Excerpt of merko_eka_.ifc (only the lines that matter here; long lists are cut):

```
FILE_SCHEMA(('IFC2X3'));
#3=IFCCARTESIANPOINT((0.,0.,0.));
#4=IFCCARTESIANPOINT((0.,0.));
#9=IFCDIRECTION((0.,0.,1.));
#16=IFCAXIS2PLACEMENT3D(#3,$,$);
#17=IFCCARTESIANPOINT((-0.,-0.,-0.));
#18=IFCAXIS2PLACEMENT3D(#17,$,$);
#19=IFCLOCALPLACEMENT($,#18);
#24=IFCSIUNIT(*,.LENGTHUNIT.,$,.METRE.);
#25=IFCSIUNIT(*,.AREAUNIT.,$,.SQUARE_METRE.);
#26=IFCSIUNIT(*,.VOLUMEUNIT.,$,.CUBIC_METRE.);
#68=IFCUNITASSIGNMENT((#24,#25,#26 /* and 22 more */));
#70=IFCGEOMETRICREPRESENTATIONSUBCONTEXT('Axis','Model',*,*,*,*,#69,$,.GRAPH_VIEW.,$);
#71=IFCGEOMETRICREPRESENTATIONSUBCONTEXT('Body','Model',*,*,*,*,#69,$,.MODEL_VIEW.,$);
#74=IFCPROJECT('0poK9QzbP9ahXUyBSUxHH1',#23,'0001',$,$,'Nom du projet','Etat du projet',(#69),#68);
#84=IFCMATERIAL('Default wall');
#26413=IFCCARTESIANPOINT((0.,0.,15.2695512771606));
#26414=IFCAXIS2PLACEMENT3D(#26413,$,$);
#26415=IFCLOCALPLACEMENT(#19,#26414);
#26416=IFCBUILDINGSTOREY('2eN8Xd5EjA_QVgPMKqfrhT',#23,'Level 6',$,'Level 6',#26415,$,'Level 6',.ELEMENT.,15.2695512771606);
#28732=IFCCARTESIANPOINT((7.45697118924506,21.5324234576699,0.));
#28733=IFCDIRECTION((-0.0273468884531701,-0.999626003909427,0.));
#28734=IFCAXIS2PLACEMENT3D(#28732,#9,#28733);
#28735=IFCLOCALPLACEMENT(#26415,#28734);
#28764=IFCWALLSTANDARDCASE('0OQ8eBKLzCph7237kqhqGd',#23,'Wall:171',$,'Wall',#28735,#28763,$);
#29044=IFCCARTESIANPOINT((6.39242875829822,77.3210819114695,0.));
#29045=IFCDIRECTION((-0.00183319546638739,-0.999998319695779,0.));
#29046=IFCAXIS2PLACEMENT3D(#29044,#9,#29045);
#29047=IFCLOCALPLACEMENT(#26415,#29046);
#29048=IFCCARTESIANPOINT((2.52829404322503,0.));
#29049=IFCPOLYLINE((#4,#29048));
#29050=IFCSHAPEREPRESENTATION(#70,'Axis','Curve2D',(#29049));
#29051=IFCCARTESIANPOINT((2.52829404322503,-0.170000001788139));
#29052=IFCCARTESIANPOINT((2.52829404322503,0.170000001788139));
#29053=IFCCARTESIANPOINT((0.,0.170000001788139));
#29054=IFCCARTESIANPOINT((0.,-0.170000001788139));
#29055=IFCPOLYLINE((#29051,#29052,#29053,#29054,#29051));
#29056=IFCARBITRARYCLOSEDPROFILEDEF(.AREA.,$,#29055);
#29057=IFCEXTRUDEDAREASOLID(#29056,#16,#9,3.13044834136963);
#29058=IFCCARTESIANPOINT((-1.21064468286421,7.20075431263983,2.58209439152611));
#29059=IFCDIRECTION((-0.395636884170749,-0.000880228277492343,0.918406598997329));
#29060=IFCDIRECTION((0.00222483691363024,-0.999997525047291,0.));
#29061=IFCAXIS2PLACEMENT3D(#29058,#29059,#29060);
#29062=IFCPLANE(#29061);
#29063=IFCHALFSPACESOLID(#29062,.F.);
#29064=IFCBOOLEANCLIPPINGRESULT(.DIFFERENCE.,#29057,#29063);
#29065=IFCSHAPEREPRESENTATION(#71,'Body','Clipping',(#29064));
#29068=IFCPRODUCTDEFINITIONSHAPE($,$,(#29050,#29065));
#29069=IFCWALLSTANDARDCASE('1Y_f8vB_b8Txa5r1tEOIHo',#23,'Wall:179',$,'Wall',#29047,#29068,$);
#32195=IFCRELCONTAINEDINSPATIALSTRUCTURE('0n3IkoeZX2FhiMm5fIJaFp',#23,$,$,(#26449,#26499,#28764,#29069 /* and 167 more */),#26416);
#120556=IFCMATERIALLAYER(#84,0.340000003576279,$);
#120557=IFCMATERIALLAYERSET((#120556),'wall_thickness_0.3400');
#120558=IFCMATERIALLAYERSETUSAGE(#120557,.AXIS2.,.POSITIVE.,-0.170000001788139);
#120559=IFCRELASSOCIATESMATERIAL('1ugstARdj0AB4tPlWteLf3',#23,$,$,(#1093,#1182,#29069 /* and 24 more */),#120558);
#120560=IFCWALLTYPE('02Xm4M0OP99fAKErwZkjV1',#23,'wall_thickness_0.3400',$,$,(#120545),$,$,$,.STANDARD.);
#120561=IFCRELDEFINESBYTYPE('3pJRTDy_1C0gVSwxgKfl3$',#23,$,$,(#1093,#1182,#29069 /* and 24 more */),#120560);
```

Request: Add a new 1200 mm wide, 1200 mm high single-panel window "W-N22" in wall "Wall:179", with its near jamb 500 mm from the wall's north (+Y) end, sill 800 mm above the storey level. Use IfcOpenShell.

```python
import numpy as np
import ifcopenshell
import ifcopenshell.api.feature
import ifcopenshell.api.geometry
import ifcopenshell.api.root
import ifcopenshell.api.spatial
import ifcopenshell.api.type
import ifcopenshell.geom
import ifcopenshell.util.element
import ifcopenshell.util.placement
import ifcopenshell.util.representation
import ifcopenshell.util.shape
import ifcopenshell.util.unit

model = ifcopenshell.open("merko_eka_.ifc")
unit_scale = ifcopenshell.util.unit.calculate_unit_scale(model)
settings = ifcopenshell.geom.settings()


def volume(element):
    """Net volume in cubic metres, openings subtracted."""
    shape = ifcopenshell.geom.create_shape(settings, element)
    return ifcopenshell.util.shape.get_volume(shape.geometry)


wall = model.by_guid("1Y_f8vB_b8Txa5r1tEOIHo")
storey = ifcopenshell.util.element.get_container(wall, ifc_class="IfcBuildingStorey")
context = ifcopenshell.util.representation.get_context(model, "Model", "Body", "MODEL_VIEW")
before = volume(wall)

width, height, from_end, sill = 1.2, 1.2, 0.5, 0.8  # metres

# The wall runs along its own X axis, and the end named is its -X end.
wall_shape = ifcopenshell.geom.create_shape(settings, wall)
x, y, z = ifcopenshell.util.shape.get_vertices(wall_shape.geometry).T
start = x.min() + from_end
face, thickness = float(y.min()), float(y.max() - y.min())
wall_matrix = ifcopenshell.util.placement.get_local_placement(wall.ObjectPlacement)
level = ifcopenshell.util.placement.get_local_placement(storey.ObjectPlacement)[2, 3]


def in_wall(x, y):
    """Placement at x, y metres in the wall's axes, at sill height."""
    matrix = wall_matrix.copy()
    matrix[:, 3] = wall_matrix @ np.array([x / unit_scale, y / unit_scale, 0.0, 1.0])
    matrix[2, 3] = level + sill / unit_scale
    return matrix


# Opening: a box that overshoots both wall faces by 50 mm.
opening = ifcopenshell.api.root.create_entity(model, ifc_class="IfcOpeningElement")
box = ifcopenshell.api.geometry.add_wall_representation(
    model, context=context, length=width, height=height, thickness=thickness + 0.1
)
ifcopenshell.api.geometry.assign_representation(model, product=opening, representation=box)
ifcopenshell.api.geometry.edit_object_placement(model, product=opening, matrix=in_wall(start, face - 0.05), is_si=False)
ifcopenshell.api.feature.add_feature(model, feature=opening, element=wall)

window = ifcopenshell.api.root.create_entity(model, ifc_class="IfcWindow", name="W-N22")
window.OverallWidth, window.OverallHeight = width / unit_scale, height / unit_scale
body = ifcopenshell.api.geometry.add_window_representation(
    model,
    context=context,
    overall_width=window.OverallWidth,
    overall_height=window.OverallHeight,
    partition_type="SINGLE_PANEL",
)
ifcopenshell.api.geometry.assign_representation(model, product=window, representation=body)
ifcopenshell.api.spatial.assign_container(model, products=[window], relating_structure=storey)
fills = ifcopenshell.api.feature.add_filling(model, opening=opening, element=window)
fills.OwnerHistory = window.OwnerHistory  # required in IFC2X3

# IFC2X3 keeps the operation on the window style.
style = ifcopenshell.api.root.create_entity(model, ifc_class="IfcWindowStyle", name="W-N22")
style.OperationType, style.ConstructionType = "SINGLE_PANEL", "NOTDEFINED"
style.ParameterTakesPrecedence = style.Sizeable = False
ifcopenshell.api.type.assign_type(model, related_objects=[window], relating_type=style)

# Centre the window in the wall's thickness.
ifcopenshell.api.geometry.edit_object_placement(model, product=window, matrix=in_wall(start, face), is_si=False)
window_shape = ifcopenshell.geom.create_shape(settings, window)
depth = ifcopenshell.util.shape.get_vertices(window_shape.geometry)[:, 1]
offset = face + thickness / 2 - (depth.min() + depth.max()) / 2
ifcopenshell.api.geometry.edit_object_placement(model, product=window, matrix=in_wall(start, offset), is_si=False)

after = volume(wall)

print(f"wall volume {before:.3f} -> {after:.3f} m3")

model.write("merko_eka__v2.ifc")
```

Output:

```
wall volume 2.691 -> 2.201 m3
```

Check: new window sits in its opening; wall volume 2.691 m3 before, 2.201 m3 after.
